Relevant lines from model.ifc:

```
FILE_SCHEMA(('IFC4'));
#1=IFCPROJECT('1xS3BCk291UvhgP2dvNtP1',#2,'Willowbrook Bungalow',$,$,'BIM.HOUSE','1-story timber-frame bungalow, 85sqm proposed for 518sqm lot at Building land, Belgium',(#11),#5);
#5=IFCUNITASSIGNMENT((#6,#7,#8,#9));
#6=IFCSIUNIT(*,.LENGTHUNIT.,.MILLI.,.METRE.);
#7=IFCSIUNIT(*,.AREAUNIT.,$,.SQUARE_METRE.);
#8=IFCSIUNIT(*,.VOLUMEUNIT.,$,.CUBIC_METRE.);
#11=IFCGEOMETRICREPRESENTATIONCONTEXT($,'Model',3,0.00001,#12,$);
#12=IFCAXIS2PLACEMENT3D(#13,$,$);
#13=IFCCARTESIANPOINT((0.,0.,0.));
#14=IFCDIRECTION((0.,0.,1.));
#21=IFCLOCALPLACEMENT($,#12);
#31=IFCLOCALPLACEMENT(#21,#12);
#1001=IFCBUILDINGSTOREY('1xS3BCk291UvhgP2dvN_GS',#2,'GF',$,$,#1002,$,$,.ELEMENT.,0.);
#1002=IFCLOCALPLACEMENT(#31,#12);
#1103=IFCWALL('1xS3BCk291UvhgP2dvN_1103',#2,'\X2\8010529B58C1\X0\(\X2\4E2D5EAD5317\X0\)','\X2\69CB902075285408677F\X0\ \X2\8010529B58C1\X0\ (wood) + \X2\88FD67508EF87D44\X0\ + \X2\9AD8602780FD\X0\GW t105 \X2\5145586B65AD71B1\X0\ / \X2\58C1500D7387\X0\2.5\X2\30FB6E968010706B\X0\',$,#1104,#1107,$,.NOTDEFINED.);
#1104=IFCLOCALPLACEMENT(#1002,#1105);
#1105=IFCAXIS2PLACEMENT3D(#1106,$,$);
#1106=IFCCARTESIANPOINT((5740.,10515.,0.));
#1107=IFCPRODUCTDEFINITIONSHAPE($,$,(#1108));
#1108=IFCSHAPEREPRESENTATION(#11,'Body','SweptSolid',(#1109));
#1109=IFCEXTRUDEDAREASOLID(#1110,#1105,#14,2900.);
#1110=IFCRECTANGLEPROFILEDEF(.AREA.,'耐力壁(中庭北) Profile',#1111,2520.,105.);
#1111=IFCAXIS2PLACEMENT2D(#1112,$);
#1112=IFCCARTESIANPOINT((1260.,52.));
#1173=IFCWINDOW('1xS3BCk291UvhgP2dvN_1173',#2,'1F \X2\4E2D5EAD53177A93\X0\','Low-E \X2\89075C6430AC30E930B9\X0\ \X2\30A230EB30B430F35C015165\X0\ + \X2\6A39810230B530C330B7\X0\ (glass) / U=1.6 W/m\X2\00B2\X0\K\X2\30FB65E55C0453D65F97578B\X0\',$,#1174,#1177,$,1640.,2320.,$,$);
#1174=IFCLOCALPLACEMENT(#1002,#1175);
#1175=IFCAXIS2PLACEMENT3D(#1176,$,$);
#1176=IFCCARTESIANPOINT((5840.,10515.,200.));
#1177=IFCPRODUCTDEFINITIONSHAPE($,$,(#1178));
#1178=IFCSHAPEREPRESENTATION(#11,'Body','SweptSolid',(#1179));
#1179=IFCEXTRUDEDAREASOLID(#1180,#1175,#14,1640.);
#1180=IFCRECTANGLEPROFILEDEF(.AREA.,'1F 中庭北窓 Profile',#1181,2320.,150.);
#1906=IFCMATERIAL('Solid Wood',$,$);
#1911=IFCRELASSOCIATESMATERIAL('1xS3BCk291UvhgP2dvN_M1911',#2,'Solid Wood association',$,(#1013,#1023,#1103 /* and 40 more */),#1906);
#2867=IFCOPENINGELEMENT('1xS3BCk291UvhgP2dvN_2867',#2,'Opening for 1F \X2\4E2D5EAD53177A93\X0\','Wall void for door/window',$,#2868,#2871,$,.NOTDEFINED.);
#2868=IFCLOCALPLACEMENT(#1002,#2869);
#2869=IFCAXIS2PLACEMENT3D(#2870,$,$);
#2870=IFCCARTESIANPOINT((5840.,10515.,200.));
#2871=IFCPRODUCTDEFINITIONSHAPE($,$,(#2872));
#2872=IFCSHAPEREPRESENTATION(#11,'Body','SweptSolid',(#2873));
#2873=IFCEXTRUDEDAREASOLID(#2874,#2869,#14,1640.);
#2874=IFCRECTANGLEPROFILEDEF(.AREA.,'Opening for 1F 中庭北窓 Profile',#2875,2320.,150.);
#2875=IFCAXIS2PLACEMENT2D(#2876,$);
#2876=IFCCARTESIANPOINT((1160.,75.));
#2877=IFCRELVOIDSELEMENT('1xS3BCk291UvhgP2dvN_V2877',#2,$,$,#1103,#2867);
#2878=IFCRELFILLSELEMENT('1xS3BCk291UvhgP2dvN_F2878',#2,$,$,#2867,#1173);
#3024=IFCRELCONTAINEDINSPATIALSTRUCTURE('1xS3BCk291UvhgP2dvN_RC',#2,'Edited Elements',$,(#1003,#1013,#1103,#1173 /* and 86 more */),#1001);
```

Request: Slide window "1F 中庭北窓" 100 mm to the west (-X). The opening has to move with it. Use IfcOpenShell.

```python
import ifcopenshell
import ifcopenshell.api.geometry
import ifcopenshell.util.placement
import ifcopenshell.util.unit

model = ifcopenshell.open("model.ifc")
unit_scale = ifcopenshell.util.unit.calculate_unit_scale(model)

window = model.by_id(1173)
opening = window.FillsVoids[0].RelatingOpeningElement
wall = opening.VoidsElements[0].RelatingBuildingElement

wall_matrix = ifcopenshell.util.placement.get_local_placement(wall.ObjectPlacement)
shift = wall_matrix[:3, 0] * -0.1 / unit_scale
before = ifcopenshell.util.placement.get_local_placement(window.ObjectPlacement)[:3, 3].copy()

# The window is not placed relative to its opening, so move both.
for product in (opening, window):
    matrix = ifcopenshell.util.placement.get_local_placement(product.ObjectPlacement)
    matrix[:3, 3] += shift
    ifcopenshell.api.geometry.edit_object_placement(model, product=product, matrix=matrix, is_si=False)

after = ifcopenshell.util.placement.get_local_placement(window.ObjectPlacement)[:3, 3]
print("window moved by", (after - before).round(3) + 0.0)

model.write("model_updated.ifc")
```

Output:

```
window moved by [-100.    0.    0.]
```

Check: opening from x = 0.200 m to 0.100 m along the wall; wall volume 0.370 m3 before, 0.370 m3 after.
